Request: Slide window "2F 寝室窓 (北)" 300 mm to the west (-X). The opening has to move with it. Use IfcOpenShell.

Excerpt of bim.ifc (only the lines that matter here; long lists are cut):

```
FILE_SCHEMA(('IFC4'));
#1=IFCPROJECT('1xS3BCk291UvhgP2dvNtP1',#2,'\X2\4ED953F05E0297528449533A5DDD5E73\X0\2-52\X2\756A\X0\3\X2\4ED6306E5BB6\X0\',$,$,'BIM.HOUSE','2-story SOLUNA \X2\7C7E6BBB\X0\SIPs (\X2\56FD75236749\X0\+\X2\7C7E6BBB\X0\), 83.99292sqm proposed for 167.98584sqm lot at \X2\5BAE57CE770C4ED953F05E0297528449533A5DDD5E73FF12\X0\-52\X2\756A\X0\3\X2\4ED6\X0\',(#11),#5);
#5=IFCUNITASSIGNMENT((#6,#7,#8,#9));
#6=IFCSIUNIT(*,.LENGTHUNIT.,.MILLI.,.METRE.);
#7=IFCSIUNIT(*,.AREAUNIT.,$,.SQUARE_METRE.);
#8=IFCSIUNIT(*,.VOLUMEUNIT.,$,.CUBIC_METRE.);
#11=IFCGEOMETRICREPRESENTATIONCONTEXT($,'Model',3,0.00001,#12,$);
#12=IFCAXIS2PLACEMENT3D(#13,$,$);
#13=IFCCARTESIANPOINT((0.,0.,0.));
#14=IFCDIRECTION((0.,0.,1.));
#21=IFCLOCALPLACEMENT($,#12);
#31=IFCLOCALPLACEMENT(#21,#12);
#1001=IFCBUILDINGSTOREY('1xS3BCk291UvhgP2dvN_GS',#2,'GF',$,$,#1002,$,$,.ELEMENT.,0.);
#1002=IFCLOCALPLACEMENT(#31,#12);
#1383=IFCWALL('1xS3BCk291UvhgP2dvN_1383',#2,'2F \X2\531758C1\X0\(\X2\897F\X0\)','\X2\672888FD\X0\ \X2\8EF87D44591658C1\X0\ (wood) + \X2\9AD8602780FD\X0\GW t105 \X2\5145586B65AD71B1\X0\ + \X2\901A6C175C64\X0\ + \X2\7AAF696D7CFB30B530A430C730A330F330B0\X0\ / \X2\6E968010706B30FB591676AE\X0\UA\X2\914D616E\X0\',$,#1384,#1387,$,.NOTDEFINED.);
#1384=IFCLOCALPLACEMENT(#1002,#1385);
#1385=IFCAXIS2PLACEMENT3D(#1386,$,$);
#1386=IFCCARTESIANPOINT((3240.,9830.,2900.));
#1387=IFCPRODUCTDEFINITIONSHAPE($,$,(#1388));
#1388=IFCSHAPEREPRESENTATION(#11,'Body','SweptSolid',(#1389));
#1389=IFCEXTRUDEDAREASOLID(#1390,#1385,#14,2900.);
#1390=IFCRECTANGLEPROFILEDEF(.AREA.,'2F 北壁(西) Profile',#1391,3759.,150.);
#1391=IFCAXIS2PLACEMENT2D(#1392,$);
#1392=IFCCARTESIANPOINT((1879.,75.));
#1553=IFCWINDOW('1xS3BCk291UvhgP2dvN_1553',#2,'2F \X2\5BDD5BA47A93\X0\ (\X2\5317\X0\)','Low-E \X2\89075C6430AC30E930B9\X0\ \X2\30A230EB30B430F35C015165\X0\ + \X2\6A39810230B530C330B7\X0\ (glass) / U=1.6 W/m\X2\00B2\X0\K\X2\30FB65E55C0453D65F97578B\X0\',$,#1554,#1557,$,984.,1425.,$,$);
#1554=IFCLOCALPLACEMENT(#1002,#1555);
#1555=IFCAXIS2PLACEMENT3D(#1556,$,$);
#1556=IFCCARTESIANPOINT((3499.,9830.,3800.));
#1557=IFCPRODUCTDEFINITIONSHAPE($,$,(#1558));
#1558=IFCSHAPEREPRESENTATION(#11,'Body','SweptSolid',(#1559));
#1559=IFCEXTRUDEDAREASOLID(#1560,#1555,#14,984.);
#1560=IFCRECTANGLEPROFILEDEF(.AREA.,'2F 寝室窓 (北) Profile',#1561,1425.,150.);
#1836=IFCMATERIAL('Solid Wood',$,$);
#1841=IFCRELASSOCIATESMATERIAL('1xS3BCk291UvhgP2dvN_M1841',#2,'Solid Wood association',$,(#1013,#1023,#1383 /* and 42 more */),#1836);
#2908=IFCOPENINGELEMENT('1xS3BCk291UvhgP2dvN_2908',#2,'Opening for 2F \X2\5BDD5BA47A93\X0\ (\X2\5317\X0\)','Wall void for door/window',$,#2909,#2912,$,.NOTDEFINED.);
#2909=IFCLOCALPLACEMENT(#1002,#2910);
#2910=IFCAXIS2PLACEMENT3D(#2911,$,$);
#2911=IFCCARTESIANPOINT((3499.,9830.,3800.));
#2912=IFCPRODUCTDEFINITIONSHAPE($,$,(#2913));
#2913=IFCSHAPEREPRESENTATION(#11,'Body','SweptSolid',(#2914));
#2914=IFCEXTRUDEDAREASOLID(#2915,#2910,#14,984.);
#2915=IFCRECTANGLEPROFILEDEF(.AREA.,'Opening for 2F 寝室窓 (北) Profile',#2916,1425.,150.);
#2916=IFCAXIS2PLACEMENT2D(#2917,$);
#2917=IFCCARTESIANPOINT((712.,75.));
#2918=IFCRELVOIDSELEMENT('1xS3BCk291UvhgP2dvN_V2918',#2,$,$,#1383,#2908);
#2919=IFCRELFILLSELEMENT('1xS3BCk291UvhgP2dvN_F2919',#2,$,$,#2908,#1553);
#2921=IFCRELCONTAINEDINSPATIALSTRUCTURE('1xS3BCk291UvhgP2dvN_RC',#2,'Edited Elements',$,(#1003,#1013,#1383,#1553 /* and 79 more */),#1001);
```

```python
import ifcopenshell
import ifcopenshell.api.geometry
import ifcopenshell.util.placement
import ifcopenshell.util.unit

model = ifcopenshell.open("bim.ifc")
unit_scale = ifcopenshell.util.unit.calculate_unit_scale(model)

window = model.by_guid("1xS3BCk291UvhgP2dvN_1553")
opening = window.FillsVoids[0].RelatingOpeningElement
wall = opening.VoidsElements[0].RelatingBuildingElement

wall_matrix = ifcopenshell.util.placement.get_local_placement(wall.ObjectPlacement)
shift = wall_matrix[:3, 0] * -0.3 / unit_scale
before = ifcopenshell.util.placement.get_local_placement(window.ObjectPlacement)[:3, 3].copy()

# The window is not placed relative to its opening, so move both.
for product in (opening, window):
    matrix = ifcopenshell.util.placement.get_local_placement(product.ObjectPlacement)
    matrix[:3, 3] += shift
    ifcopenshell.api.geometry.edit_object_placement(model, product=product, matrix=matrix, is_si=False)

after = ifcopenshell.util.placement.get_local_placement(window.ObjectPlacement)[:3, 3]
print("window moved by", (after - before).round(3) + 0.0)

model.write("bim-out.ifc")
```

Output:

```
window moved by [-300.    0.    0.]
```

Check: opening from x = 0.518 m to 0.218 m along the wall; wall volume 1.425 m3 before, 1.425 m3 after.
